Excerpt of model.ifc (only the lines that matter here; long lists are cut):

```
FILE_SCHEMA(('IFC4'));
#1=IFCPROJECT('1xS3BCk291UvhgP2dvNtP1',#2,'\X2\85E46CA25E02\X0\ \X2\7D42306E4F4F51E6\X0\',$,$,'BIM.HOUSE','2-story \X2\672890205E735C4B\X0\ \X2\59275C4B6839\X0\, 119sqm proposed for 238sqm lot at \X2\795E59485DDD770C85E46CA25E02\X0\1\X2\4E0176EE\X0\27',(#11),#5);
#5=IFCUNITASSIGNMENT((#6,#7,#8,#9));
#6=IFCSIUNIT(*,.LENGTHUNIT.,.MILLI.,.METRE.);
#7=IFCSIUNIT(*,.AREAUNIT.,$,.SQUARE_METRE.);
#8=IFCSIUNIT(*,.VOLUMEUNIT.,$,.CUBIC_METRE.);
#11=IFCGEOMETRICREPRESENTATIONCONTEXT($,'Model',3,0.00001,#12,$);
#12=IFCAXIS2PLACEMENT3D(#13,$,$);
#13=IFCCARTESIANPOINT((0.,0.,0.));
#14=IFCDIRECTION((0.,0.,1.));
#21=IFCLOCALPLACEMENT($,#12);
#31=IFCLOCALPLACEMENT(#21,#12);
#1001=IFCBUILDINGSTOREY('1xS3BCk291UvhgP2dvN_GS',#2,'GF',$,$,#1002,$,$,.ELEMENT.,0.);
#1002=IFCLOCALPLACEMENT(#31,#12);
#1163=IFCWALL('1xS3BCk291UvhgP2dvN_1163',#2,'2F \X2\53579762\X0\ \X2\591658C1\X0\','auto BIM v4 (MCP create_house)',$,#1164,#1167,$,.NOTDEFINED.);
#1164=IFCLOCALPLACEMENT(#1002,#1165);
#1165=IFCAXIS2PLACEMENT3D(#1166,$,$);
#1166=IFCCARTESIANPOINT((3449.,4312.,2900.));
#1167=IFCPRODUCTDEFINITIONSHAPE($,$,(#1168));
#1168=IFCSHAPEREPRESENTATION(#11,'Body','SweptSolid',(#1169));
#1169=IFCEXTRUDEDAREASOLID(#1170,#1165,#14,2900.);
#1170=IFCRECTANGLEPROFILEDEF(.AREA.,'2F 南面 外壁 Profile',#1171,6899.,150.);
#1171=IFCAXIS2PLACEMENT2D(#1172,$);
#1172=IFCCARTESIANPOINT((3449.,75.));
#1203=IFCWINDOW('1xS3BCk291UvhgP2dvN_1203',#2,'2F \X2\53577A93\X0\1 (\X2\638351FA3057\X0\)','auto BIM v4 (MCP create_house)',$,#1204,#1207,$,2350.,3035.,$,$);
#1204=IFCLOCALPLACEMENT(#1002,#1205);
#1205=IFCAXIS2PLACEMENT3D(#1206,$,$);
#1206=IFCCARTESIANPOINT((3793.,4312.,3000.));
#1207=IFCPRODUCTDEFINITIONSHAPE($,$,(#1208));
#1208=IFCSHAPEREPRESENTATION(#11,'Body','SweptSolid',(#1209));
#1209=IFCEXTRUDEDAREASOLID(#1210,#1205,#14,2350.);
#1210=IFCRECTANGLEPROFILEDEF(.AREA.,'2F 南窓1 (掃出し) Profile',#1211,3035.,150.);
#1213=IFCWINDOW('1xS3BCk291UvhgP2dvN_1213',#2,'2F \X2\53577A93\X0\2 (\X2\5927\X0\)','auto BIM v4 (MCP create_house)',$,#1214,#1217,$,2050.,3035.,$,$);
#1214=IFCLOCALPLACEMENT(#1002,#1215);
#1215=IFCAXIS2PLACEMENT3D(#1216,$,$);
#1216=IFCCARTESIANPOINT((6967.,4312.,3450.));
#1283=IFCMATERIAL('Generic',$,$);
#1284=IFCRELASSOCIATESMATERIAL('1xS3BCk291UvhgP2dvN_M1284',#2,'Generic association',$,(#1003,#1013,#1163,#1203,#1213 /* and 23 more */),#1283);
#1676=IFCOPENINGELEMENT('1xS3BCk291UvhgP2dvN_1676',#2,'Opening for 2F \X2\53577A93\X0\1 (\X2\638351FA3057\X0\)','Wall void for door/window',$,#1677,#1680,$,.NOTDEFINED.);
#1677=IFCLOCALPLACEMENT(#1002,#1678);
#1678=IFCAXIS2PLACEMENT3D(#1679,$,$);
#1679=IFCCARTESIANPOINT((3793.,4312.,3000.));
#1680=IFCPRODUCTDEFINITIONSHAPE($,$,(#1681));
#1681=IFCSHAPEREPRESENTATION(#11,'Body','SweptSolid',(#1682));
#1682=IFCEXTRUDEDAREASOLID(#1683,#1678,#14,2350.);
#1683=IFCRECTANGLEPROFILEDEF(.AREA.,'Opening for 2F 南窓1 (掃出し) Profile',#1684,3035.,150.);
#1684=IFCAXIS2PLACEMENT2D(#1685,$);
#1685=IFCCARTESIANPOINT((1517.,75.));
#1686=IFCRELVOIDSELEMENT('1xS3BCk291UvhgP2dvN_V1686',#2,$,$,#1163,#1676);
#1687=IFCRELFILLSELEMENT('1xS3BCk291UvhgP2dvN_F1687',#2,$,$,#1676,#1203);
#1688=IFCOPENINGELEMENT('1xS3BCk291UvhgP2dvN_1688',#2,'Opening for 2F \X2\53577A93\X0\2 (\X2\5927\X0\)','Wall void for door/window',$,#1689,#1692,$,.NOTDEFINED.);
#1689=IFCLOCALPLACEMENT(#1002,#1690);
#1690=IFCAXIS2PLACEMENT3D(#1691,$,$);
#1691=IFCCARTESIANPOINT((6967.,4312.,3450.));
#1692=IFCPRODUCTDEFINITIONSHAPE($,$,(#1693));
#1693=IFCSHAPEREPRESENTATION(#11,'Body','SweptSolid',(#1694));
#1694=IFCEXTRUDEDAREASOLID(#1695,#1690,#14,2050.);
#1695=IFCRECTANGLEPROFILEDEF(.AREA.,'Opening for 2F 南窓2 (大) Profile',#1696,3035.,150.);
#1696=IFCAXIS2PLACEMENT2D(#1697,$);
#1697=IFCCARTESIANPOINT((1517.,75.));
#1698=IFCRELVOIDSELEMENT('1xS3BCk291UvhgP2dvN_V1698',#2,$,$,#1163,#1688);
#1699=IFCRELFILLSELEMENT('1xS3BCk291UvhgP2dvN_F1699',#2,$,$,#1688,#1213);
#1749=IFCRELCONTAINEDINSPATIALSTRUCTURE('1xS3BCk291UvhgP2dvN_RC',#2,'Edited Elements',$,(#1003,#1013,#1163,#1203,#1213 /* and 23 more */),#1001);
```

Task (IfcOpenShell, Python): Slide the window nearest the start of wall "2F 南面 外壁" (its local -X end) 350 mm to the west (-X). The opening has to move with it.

```python
import ifcopenshell
import ifcopenshell.api.geometry
import ifcopenshell.util.placement

model = ifcopenshell.open("model.ifc")

window = model.by_guid("1xS3BCk291UvhgP2dvN_1203")
opening = window.FillsVoids[0].RelatingOpeningElement
wall = opening.VoidsElements[0].RelatingBuildingElement

wall_matrix = ifcopenshell.util.placement.get_local_placement(wall.ObjectPlacement)
shift = wall_matrix[:3, 0] * -350.0
before = ifcopenshell.util.placement.get_local_placement(window.ObjectPlacement)[:3, 3].copy()

# The window is not placed relative to its opening, so move both.
for product in (opening, window):
    matrix = ifcopenshell.util.placement.get_local_placement(product.ObjectPlacement)
    matrix[:3, 3] += shift
    ifcopenshell.api.geometry.edit_object_placement(model, product=product, matrix=matrix, is_si=False)

after = ifcopenshell.util.placement.get_local_placement(window.ObjectPlacement)[:3, 3]
print("window moved by", (after - before).round(3) + 0.0)

model.write("model-out.ifc")
```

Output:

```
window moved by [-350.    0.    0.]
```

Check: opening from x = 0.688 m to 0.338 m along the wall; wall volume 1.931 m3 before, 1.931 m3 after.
